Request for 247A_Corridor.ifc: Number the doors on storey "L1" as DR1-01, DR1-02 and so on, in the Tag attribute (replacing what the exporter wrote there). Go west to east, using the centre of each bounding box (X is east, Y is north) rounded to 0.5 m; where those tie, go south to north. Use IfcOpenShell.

First a look at what the model holds.

```python
import ifcopenshell
import ifcopenshell.util.element
import ifcopenshell.util.placement

model = ifcopenshell.open("247A_Corridor.ifc")
print(model.schema)
storey = next(s for s in model.by_type("IfcBuildingStorey") if s.Name == "L1")
doors = [e for e in ifcopenshell.util.element.get_decomposition(storey) if e.is_a("IfcDoor")]
for e in sorted(doors, key=lambda e: e.id()):
    origin = ifcopenshell.util.placement.get_local_placement(e.ObjectPlacement)[:3, 3]
    print(e.id(), e.Tag, e.Name, origin.round(2) + 0.0, sep=" | ")
```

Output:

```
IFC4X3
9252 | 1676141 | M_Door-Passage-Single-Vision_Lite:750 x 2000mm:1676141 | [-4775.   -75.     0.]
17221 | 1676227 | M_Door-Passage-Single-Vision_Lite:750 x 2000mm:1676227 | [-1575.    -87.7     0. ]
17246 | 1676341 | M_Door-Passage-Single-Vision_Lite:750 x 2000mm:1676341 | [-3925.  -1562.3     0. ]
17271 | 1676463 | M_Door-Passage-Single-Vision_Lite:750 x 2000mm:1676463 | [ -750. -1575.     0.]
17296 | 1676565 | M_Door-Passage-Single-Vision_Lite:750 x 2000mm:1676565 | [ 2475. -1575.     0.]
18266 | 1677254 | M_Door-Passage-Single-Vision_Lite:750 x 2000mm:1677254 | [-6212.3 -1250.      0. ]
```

```python
import ifcopenshell
import ifcopenshell.geom
import ifcopenshell.util.element
import ifcopenshell.util.shape

model = ifcopenshell.open("247A_Corridor.ifc")
settings = ifcopenshell.geom.settings()
settings.set("use-world-coords", True)


def centre(element):
    shape = ifcopenshell.geom.create_shape(settings, element)
    return ifcopenshell.util.shape.get_bbox_centroid(shape.geometry)


storey = next(s for s in model.by_type("IfcBuildingStorey") if s.Name == "L1")
doors = [e for e in ifcopenshell.util.element.get_decomposition(storey) if e.is_a("IfcDoor")]

# Insertion points can sit at a corner or the storey origin, so sort by the geometry (in metres).
centres = {e: centre(e) for e in doors}
doors.sort(key=lambda e: (round(centres[e][0] / 0.5), centres[e][1]))

for i, e in enumerate(doors, start=1):
    number = f"DR1-{i:02d}"
    e.Tag = number
    print(e.id(), number)

model.write("247A_Corridor_updated.ifc")
```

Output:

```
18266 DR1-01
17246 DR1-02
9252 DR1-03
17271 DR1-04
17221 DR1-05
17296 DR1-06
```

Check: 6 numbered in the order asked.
